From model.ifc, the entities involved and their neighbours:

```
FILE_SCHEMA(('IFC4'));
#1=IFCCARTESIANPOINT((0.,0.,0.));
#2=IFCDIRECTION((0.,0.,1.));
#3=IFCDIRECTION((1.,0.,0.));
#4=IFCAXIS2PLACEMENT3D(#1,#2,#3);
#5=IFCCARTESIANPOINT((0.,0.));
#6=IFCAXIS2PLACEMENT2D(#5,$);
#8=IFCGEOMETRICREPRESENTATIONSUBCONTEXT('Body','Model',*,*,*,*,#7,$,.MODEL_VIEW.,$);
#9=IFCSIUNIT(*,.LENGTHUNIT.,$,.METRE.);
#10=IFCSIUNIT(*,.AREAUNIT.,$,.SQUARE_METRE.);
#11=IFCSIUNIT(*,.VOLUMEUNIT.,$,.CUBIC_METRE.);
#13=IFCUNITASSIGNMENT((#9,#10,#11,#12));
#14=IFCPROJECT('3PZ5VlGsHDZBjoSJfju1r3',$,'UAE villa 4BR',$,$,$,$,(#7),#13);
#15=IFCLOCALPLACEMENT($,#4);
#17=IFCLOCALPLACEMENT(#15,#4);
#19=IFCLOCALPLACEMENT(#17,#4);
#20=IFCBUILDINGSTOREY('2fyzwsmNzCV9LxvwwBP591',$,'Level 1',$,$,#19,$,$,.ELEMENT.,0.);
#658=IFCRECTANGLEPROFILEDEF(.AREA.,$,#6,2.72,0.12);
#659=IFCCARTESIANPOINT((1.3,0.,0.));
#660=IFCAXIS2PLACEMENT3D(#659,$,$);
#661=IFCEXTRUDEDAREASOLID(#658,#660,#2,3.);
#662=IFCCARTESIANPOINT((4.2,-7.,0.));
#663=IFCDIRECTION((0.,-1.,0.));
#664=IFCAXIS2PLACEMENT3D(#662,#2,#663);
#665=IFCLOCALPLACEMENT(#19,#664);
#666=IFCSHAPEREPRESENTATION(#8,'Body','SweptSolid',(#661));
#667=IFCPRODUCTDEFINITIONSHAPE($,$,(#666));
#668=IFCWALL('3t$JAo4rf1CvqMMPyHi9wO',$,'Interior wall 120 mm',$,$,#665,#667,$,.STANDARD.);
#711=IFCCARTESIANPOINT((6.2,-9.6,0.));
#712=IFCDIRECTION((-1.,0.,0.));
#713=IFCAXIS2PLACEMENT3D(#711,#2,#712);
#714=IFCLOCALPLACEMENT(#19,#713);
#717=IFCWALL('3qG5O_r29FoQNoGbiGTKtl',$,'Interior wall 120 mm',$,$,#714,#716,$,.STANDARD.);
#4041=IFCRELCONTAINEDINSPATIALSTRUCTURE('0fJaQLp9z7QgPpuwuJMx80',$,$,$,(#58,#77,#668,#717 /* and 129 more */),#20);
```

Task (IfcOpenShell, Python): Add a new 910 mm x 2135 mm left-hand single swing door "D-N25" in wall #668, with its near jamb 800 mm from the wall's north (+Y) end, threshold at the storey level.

```python
import numpy as np
import ifcopenshell
import ifcopenshell.api.feature
import ifcopenshell.api.geometry
import ifcopenshell.api.root
import ifcopenshell.api.spatial
import ifcopenshell.geom
import ifcopenshell.util.element
import ifcopenshell.util.placement
import ifcopenshell.util.representation
import ifcopenshell.util.shape
import ifcopenshell.util.unit

model = ifcopenshell.open("model.ifc")
unit_scale = ifcopenshell.util.unit.calculate_unit_scale(model)
settings = ifcopenshell.geom.settings()


def volume(element):
    """Net volume in cubic metres, openings subtracted."""
    shape = ifcopenshell.geom.create_shape(settings, element)
    return ifcopenshell.util.shape.get_volume(shape.geometry)


wall = model.by_guid("3t$JAo4rf1CvqMMPyHi9wO")
storey = ifcopenshell.util.element.get_container(wall, ifc_class="IfcBuildingStorey")
context = ifcopenshell.util.representation.get_context(model, "Model", "Body", "MODEL_VIEW")
before = volume(wall)

width, height, from_end, sill = 0.91, 2.135, 0.8, 0.0  # metres

# The wall runs along its own X axis, and the end named is its -X end.
wall_shape = ifcopenshell.geom.create_shape(settings, wall)
x, y, z = ifcopenshell.util.shape.get_vertices(wall_shape.geometry).T
start = x.min() + from_end
face, thickness = float(y.min()), float(y.max() - y.min())
wall_matrix = ifcopenshell.util.placement.get_local_placement(wall.ObjectPlacement)
level = ifcopenshell.util.placement.get_local_placement(storey.ObjectPlacement)[2, 3]


def in_wall(x, y):
    """Placement at x, y metres in the wall's axes, at sill height."""
    matrix = wall_matrix.copy()
    matrix[:, 3] = wall_matrix @ np.array([x / unit_scale, y / unit_scale, 0.0, 1.0])
    matrix[2, 3] = level + sill / unit_scale
    return matrix


# Opening: a box that overshoots both wall faces by 50 mm.
opening = ifcopenshell.api.root.create_entity(model, ifc_class="IfcOpeningElement", predefined_type="OPENING")
box = ifcopenshell.api.geometry.add_wall_representation(
    model, context=context, length=width, height=height, thickness=thickness + 0.1
)
ifcopenshell.api.geometry.assign_representation(model, product=opening, representation=box)
ifcopenshell.api.geometry.edit_object_placement(model, product=opening, matrix=in_wall(start, face - 0.05), is_si=False)
ifcopenshell.api.feature.add_feature(model, feature=opening, element=wall)

door = ifcopenshell.api.root.create_entity(model, ifc_class="IfcDoor", name="D-N25", predefined_type="DOOR")
door.OverallWidth, door.OverallHeight = width / unit_scale, height / unit_scale
door.OperationType = "SINGLE_SWING_LEFT"
body = ifcopenshell.api.geometry.add_door_representation(
    model,
    context=context,
    overall_width=door.OverallWidth,
    overall_height=door.OverallHeight,
    operation_type="SINGLE_SWING_LEFT",
    lining_properties={"LiningDepth": thickness / unit_scale, "ThresholdDepth": thickness / unit_scale},
)
ifcopenshell.api.geometry.assign_representation(model, product=door, representation=body)
ifcopenshell.api.spatial.assign_container(model, products=[door], relating_structure=storey)
ifcopenshell.api.feature.add_filling(model, opening=opening, element=door)

# The lining spans the wall, so the door starts at the wall face.
ifcopenshell.api.geometry.edit_object_placement(model, product=door, matrix=in_wall(start, face), is_si=False)

after = volume(wall)

print(f"wall volume {before:.3f} -> {after:.3f} m3")

model.write("model_edited.ifc")
```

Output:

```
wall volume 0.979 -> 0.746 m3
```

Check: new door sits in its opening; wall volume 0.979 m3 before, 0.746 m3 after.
